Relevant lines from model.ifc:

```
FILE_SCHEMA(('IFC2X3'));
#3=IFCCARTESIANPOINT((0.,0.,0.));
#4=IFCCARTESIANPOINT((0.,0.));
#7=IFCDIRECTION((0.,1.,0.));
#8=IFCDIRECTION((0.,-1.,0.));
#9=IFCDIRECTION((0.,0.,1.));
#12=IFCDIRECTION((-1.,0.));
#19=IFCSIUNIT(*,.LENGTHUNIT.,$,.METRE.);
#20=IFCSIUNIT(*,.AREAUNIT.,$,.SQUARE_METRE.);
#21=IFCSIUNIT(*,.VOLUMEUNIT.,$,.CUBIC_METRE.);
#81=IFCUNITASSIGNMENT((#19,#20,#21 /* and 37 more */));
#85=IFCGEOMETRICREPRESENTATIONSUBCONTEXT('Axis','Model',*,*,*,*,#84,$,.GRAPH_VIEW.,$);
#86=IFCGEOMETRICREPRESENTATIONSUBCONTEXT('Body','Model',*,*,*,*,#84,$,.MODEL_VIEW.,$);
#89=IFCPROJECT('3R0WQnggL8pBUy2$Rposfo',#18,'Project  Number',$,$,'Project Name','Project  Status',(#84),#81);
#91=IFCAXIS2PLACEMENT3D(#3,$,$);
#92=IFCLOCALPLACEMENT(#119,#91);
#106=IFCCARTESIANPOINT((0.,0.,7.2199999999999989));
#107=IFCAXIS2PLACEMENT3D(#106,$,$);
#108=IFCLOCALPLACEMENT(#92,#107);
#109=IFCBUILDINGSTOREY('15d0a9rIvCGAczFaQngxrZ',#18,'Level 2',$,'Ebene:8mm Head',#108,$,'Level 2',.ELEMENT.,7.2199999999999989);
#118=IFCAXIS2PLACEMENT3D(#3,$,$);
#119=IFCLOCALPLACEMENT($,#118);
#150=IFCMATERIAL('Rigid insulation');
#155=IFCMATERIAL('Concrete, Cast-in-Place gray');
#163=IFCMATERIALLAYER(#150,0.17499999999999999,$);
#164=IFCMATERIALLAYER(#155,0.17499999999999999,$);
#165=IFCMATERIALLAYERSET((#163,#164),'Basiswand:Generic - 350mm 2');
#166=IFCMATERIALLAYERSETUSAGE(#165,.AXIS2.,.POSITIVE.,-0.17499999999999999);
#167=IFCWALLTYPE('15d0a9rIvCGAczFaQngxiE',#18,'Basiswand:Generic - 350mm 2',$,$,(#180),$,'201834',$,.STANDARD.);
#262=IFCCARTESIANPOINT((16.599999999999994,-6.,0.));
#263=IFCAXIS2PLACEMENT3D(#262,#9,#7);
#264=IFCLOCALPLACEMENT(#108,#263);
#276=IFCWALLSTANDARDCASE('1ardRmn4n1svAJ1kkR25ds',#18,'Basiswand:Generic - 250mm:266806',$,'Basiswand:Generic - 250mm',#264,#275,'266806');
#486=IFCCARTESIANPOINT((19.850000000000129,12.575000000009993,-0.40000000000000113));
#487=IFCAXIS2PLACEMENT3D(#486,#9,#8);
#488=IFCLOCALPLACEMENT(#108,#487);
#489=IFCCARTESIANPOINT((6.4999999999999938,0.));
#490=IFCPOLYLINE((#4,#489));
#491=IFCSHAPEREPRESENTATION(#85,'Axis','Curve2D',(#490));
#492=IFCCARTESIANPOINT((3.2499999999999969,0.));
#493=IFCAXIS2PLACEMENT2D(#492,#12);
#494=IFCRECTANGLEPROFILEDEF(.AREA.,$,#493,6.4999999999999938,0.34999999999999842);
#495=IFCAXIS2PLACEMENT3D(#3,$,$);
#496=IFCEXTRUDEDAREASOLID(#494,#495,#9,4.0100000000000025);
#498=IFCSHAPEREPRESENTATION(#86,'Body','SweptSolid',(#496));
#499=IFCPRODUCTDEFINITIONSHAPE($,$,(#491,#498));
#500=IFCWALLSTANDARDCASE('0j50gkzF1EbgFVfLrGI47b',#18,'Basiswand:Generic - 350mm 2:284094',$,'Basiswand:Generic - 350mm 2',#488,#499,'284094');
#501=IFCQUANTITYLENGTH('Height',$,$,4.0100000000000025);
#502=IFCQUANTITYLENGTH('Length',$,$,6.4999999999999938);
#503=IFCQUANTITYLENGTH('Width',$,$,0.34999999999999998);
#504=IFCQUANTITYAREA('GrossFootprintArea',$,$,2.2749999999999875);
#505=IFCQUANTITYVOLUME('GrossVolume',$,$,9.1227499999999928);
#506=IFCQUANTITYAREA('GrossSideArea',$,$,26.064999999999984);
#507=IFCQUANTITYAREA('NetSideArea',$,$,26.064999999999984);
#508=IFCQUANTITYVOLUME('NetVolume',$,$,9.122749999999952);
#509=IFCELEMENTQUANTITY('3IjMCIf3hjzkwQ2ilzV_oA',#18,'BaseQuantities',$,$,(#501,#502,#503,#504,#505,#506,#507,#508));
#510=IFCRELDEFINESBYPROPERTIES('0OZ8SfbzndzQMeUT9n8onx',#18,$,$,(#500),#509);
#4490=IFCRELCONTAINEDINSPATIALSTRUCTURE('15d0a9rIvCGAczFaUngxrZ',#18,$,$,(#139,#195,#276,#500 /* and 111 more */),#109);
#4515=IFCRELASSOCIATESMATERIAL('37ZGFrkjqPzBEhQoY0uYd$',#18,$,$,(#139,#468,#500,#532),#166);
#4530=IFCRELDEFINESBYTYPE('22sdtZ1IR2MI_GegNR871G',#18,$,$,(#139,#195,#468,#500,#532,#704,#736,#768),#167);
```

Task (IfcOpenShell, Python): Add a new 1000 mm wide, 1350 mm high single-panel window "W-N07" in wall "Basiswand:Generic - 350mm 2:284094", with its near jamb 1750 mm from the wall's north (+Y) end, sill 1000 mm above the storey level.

```python
import numpy as np
import ifcopenshell
import ifcopenshell.api.feature
import ifcopenshell.api.geometry
import ifcopenshell.api.pset
import ifcopenshell.api.root
import ifcopenshell.api.spatial
import ifcopenshell.api.type
import ifcopenshell.geom
import ifcopenshell.util.element
import ifcopenshell.util.placement
import ifcopenshell.util.representation
import ifcopenshell.util.shape
import ifcopenshell.util.unit

model = ifcopenshell.open("model.ifc")
unit_scale = ifcopenshell.util.unit.calculate_unit_scale(model)
area_scale = ifcopenshell.util.unit.calculate_unit_scale(model, "AREAUNIT")
volume_scale = ifcopenshell.util.unit.calculate_unit_scale(model, "VOLUMEUNIT")
settings = ifcopenshell.geom.settings()


def volume(element):
    """Net volume in cubic metres, openings subtracted."""
    shape = ifcopenshell.geom.create_shape(settings, element)
    return ifcopenshell.util.shape.get_volume(shape.geometry)


wall = model.by_guid("0j50gkzF1EbgFVfLrGI47b")
storey = ifcopenshell.util.element.get_container(wall, ifc_class="IfcBuildingStorey")
context = ifcopenshell.util.representation.get_context(model, "Model", "Body", "MODEL_VIEW")
before = volume(wall)

width, height, from_end, sill = 1, 1.35, 1.75, 1  # metres

# The wall runs along its own X axis, and the end named is its -X end.
wall_shape = ifcopenshell.geom.create_shape(settings, wall)
x, y, z = ifcopenshell.util.shape.get_vertices(wall_shape.geometry).T
start = x.min() + from_end
face, thickness = float(y.min()), float(y.max() - y.min())
wall_matrix = ifcopenshell.util.placement.get_local_placement(wall.ObjectPlacement)
level = ifcopenshell.util.placement.get_local_placement(storey.ObjectPlacement)[2, 3]


def in_wall(x, y):
    """Placement at x, y metres in the wall's axes, at sill height."""
    matrix = wall_matrix.copy()
    matrix[:, 3] = wall_matrix @ np.array([x / unit_scale, y / unit_scale, 0.0, 1.0])
    matrix[2, 3] = level + sill / unit_scale
    return matrix


# Opening: a box that overshoots both wall faces by 50 mm.
opening = ifcopenshell.api.root.create_entity(model, ifc_class="IfcOpeningElement")
box = ifcopenshell.api.geometry.add_wall_representation(
    model, context=context, length=width, height=height, thickness=thickness + 0.1
)
ifcopenshell.api.geometry.assign_representation(model, product=opening, representation=box)
ifcopenshell.api.geometry.edit_object_placement(model, product=opening, matrix=in_wall(start, face - 0.05), is_si=False)
ifcopenshell.api.feature.add_feature(model, feature=opening, element=wall)

window = ifcopenshell.api.root.create_entity(model, ifc_class="IfcWindow", name="W-N07")
window.OverallWidth, window.OverallHeight = width / unit_scale, height / unit_scale
body = ifcopenshell.api.geometry.add_window_representation(
    model,
    context=context,
    overall_width=window.OverallWidth,
    overall_height=window.OverallHeight,
    partition_type="SINGLE_PANEL",
)
ifcopenshell.api.geometry.assign_representation(model, product=window, representation=body)
ifcopenshell.api.spatial.assign_container(model, products=[window], relating_structure=storey)
fills = ifcopenshell.api.feature.add_filling(model, opening=opening, element=window)
fills.OwnerHistory = window.OwnerHistory  # required in IFC2X3

# IFC2X3 keeps the operation on the window style.
style = ifcopenshell.api.root.create_entity(model, ifc_class="IfcWindowStyle", name="W-N07")
style.OperationType, style.ConstructionType = "SINGLE_PANEL", "NOTDEFINED"
style.ParameterTakesPrecedence = style.Sizeable = False
ifcopenshell.api.type.assign_type(model, related_objects=[window], relating_type=style)

# Centre the window in the wall's thickness.
ifcopenshell.api.geometry.edit_object_placement(model, product=window, matrix=in_wall(start, face), is_si=False)
window_shape = ifcopenshell.geom.create_shape(settings, window)
depth = ifcopenshell.util.shape.get_vertices(window_shape.geometry)[:, 1]
offset = face + thickness / 2 - (depth.min() + depth.max()) / 2
ifcopenshell.api.geometry.edit_object_placement(model, product=window, matrix=in_wall(start, offset), is_si=False)

after = volume(wall)

# Update the wall's stored quantities.
qto = model.by_id(ifcopenshell.util.element.get_pset(wall, "BaseQuantities", should_inherit=False)["id"])
ifcopenshell.api.pset.edit_qto(model, qto=qto, properties={
    "NetSideArea": after / thickness / area_scale,
    "NetVolume": after / volume_scale,
})

print(f"wall volume {before:.3f} -> {after:.3f} m3")

model.write("model-out.ifc")
```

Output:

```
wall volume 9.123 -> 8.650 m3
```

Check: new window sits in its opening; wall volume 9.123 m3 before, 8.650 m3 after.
